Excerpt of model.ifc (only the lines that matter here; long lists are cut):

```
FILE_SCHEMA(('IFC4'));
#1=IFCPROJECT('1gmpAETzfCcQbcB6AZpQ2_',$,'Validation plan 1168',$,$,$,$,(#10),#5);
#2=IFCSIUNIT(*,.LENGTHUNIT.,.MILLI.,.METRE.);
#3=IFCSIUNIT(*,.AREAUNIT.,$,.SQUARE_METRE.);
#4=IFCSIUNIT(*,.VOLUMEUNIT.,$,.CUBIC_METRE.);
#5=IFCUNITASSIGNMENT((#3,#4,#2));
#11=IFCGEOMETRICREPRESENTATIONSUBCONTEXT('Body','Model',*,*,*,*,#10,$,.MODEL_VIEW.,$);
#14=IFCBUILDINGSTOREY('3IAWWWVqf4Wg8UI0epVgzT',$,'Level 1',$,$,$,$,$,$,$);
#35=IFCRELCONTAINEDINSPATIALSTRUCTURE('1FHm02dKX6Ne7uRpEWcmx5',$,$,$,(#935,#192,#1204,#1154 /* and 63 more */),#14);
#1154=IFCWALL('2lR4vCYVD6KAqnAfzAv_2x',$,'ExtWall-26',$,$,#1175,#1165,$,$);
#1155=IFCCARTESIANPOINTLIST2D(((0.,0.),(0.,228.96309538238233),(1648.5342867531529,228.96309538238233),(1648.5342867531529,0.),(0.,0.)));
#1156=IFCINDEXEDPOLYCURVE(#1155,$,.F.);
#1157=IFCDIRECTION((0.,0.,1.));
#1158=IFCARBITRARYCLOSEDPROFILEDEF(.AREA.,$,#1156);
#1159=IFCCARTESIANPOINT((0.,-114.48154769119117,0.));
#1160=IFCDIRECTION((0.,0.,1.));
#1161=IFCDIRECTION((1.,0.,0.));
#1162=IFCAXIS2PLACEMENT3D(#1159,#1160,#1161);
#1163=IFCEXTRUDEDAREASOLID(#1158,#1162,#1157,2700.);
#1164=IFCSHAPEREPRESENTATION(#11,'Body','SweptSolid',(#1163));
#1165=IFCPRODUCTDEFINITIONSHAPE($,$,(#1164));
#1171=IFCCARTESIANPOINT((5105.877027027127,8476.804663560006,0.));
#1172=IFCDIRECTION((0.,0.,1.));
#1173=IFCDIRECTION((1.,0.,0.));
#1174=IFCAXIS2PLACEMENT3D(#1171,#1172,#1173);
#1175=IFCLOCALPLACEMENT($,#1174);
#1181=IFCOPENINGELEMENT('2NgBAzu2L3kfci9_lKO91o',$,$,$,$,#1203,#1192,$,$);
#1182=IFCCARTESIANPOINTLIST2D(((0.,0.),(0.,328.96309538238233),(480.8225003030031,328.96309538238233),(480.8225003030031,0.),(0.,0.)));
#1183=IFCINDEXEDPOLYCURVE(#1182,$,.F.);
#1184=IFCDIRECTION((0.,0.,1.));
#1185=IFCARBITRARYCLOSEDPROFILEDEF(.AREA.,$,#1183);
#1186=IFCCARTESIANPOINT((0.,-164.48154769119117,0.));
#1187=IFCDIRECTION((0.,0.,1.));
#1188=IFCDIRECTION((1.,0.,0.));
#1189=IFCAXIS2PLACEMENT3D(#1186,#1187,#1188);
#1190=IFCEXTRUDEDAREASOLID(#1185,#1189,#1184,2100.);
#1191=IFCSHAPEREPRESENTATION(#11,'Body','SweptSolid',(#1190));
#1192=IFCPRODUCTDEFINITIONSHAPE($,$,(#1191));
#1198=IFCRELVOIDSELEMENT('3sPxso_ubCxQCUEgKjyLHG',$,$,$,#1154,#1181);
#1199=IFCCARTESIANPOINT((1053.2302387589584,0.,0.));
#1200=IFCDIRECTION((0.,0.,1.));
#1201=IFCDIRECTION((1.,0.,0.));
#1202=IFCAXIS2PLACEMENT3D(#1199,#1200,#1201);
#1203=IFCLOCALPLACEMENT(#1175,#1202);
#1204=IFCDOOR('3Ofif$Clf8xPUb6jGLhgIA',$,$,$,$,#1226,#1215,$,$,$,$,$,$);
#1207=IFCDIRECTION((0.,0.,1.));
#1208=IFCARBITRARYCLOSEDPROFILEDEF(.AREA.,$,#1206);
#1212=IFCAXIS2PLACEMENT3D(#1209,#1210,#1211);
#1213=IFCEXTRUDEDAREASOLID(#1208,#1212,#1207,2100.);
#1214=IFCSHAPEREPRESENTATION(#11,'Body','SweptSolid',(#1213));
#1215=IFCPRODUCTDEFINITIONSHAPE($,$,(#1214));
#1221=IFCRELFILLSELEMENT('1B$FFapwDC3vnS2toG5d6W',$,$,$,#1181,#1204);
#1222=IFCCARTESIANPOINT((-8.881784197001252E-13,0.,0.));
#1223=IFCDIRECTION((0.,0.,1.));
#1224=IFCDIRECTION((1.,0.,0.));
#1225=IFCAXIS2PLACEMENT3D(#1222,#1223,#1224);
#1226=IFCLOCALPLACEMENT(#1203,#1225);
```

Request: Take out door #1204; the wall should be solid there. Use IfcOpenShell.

```python
import ifcopenshell
import ifcopenshell.api.feature
import ifcopenshell.api.root
import ifcopenshell.geom
import ifcopenshell.util.shape

model = ifcopenshell.open("model.ifc")
settings = ifcopenshell.geom.settings()


def volume(element):
    """Net volume in cubic metres, openings subtracted."""
    shape = ifcopenshell.geom.create_shape(settings, element)
    return ifcopenshell.util.shape.get_volume(shape.geometry)


door = model.by_guid("3Ofif$Clf8xPUb6jGLhgIA")
opening = door.FillsVoids[0].RelatingOpeningElement
wall = opening.VoidsElements[0].RelatingBuildingElement
before = volume(wall)

ifcopenshell.api.root.remove_product(model, product=door)
ifcopenshell.api.feature.remove_feature(model, feature=opening)

after = volume(wall)

print(f"wall volume {before:.3f} -> {after:.3f} m3")

model.write("model_v2.ifc")
```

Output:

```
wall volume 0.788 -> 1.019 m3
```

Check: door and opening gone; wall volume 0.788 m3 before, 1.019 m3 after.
